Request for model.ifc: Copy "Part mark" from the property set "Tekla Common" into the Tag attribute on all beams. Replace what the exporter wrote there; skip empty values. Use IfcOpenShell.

First a look at what the model holds.

```python
import ifcopenshell
import ifcopenshell.util.element

model = ifcopenshell.open("model.ifc")
print(model.schema)
beams = model.by_type("IfcBeam")
print(len(beams), "beams")
for e in beams[:8]:
    source = ifcopenshell.util.element.get_pset(e, "Tekla Common", "Part mark")
    target = e.Tag
    print(e.id(), repr(source), repr(target), sep=" | ")
```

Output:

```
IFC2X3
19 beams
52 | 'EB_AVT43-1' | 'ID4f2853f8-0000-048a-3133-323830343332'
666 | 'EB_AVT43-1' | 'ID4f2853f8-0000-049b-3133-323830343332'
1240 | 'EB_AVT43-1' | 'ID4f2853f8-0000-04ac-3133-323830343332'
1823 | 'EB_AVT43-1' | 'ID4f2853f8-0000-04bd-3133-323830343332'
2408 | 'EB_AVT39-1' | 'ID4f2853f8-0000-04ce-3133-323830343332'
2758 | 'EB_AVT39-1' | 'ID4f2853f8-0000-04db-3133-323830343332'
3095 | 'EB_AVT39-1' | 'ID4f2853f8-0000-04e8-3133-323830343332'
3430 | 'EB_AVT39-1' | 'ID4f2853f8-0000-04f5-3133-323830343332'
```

```python
import ifcopenshell
import ifcopenshell.util.element

model = ifcopenshell.open("model.ifc")

count = 0
for e in model.by_type("IfcBeam"):
    value = ifcopenshell.util.element.get_pset(e, "Tekla Common", "Part mark")
    current = e.Tag
    if not value or not value.strip() or current == value:
        continue
    e.Tag = value
    count += 1

print(count, "beams updated")

model.write("model_v2.ifc")
```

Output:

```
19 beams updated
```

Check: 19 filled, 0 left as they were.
